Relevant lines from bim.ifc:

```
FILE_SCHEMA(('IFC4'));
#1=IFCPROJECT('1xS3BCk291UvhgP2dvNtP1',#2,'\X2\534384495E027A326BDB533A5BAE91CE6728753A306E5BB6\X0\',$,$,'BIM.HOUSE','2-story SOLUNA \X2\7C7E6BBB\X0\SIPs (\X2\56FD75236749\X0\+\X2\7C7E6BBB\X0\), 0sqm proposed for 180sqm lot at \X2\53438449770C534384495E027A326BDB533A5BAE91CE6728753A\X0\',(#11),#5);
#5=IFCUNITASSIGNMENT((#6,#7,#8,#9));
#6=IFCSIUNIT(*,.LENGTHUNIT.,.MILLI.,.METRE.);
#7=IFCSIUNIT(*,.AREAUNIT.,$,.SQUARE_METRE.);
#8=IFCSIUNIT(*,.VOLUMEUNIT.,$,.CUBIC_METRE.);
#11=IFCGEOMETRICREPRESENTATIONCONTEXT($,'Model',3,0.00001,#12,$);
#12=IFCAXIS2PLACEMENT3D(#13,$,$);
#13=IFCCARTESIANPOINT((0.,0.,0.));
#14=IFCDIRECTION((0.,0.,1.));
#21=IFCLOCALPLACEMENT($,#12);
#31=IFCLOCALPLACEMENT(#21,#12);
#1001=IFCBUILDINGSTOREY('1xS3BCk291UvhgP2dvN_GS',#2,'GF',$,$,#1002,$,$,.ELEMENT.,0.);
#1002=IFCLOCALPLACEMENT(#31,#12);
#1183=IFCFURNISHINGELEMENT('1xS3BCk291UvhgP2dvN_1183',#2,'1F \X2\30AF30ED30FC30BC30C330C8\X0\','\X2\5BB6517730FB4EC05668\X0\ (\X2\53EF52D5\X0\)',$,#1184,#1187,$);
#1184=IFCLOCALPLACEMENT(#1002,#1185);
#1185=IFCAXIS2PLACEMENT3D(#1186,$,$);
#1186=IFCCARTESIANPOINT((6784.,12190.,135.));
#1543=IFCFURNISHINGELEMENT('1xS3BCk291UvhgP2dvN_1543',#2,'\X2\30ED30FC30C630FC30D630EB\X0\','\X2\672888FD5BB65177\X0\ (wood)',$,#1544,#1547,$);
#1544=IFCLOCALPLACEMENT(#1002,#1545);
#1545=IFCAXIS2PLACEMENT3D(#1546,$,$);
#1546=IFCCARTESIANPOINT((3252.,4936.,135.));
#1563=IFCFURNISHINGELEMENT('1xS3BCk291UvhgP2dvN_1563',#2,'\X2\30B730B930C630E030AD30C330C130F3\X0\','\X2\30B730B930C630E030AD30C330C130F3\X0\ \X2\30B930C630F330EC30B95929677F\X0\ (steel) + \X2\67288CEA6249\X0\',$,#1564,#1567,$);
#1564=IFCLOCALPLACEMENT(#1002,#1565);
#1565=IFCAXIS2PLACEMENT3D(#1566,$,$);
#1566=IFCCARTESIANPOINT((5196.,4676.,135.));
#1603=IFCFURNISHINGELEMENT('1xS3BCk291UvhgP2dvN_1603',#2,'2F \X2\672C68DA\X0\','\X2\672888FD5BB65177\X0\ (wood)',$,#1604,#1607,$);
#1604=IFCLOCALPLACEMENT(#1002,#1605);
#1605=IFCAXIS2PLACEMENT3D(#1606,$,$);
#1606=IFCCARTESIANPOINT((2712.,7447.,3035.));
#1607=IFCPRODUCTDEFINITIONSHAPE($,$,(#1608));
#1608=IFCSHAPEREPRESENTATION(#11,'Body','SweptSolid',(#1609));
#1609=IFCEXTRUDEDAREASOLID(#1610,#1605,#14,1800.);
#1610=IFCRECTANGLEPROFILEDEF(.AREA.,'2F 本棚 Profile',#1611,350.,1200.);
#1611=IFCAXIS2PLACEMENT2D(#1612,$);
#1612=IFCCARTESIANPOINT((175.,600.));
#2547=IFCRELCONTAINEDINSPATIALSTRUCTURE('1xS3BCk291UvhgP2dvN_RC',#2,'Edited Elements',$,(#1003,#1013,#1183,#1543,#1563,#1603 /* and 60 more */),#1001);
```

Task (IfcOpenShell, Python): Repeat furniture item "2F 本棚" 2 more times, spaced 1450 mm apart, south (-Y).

```python
import numpy as np
import ifcopenshell
import ifcopenshell.api.geometry
import ifcopenshell.api.root
import ifcopenshell.util.element
import ifcopenshell.util.placement
import ifcopenshell.util.unit

model = ifcopenshell.open("bim.ifc")
unit_scale = ifcopenshell.util.unit.calculate_unit_scale(model)


def reuse_history(source, copy):
    """copy_class also copies each property set's owner history, people and application; keep the originals."""
    for rel in copy.IsDefinedBy:
        if rel.is_a("IfcRelDefinesByProperties") and (history := rel.RelatingPropertyDefinition.OwnerHistory):
            rel.RelatingPropertyDefinition.OwnerHistory = source.OwnerHistory
            ifcopenshell.util.element.remove_deep2(model, history)


source = model.by_guid("1xS3BCk291UvhgP2dvN_1603")
base = ifcopenshell.util.placement.get_local_placement(source.ObjectPlacement)
step = np.array([0.0, -1.0, 0.0]) * 1.45 / unit_scale

for i in range(1, 3):
    copy = ifcopenshell.api.root.copy_class(model, product=source)
    copy.Representation = ifcopenshell.util.element.copy_deep(
        model, source.Representation, exclude=["IfcGeometricRepresentationContext", "IfcRepresentationMap"]
    )
    reuse_history(source, copy)
    matrix = base.copy()
    matrix[:3, 3] += i * step
    print("added at", matrix[:3, 3].round(3) + 0.0)
    ifcopenshell.api.geometry.edit_object_placement(model, product=copy, matrix=matrix, is_si=False)

model.write("bim_edited.ifc")
```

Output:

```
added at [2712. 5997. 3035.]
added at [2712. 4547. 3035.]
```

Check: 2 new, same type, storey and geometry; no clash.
